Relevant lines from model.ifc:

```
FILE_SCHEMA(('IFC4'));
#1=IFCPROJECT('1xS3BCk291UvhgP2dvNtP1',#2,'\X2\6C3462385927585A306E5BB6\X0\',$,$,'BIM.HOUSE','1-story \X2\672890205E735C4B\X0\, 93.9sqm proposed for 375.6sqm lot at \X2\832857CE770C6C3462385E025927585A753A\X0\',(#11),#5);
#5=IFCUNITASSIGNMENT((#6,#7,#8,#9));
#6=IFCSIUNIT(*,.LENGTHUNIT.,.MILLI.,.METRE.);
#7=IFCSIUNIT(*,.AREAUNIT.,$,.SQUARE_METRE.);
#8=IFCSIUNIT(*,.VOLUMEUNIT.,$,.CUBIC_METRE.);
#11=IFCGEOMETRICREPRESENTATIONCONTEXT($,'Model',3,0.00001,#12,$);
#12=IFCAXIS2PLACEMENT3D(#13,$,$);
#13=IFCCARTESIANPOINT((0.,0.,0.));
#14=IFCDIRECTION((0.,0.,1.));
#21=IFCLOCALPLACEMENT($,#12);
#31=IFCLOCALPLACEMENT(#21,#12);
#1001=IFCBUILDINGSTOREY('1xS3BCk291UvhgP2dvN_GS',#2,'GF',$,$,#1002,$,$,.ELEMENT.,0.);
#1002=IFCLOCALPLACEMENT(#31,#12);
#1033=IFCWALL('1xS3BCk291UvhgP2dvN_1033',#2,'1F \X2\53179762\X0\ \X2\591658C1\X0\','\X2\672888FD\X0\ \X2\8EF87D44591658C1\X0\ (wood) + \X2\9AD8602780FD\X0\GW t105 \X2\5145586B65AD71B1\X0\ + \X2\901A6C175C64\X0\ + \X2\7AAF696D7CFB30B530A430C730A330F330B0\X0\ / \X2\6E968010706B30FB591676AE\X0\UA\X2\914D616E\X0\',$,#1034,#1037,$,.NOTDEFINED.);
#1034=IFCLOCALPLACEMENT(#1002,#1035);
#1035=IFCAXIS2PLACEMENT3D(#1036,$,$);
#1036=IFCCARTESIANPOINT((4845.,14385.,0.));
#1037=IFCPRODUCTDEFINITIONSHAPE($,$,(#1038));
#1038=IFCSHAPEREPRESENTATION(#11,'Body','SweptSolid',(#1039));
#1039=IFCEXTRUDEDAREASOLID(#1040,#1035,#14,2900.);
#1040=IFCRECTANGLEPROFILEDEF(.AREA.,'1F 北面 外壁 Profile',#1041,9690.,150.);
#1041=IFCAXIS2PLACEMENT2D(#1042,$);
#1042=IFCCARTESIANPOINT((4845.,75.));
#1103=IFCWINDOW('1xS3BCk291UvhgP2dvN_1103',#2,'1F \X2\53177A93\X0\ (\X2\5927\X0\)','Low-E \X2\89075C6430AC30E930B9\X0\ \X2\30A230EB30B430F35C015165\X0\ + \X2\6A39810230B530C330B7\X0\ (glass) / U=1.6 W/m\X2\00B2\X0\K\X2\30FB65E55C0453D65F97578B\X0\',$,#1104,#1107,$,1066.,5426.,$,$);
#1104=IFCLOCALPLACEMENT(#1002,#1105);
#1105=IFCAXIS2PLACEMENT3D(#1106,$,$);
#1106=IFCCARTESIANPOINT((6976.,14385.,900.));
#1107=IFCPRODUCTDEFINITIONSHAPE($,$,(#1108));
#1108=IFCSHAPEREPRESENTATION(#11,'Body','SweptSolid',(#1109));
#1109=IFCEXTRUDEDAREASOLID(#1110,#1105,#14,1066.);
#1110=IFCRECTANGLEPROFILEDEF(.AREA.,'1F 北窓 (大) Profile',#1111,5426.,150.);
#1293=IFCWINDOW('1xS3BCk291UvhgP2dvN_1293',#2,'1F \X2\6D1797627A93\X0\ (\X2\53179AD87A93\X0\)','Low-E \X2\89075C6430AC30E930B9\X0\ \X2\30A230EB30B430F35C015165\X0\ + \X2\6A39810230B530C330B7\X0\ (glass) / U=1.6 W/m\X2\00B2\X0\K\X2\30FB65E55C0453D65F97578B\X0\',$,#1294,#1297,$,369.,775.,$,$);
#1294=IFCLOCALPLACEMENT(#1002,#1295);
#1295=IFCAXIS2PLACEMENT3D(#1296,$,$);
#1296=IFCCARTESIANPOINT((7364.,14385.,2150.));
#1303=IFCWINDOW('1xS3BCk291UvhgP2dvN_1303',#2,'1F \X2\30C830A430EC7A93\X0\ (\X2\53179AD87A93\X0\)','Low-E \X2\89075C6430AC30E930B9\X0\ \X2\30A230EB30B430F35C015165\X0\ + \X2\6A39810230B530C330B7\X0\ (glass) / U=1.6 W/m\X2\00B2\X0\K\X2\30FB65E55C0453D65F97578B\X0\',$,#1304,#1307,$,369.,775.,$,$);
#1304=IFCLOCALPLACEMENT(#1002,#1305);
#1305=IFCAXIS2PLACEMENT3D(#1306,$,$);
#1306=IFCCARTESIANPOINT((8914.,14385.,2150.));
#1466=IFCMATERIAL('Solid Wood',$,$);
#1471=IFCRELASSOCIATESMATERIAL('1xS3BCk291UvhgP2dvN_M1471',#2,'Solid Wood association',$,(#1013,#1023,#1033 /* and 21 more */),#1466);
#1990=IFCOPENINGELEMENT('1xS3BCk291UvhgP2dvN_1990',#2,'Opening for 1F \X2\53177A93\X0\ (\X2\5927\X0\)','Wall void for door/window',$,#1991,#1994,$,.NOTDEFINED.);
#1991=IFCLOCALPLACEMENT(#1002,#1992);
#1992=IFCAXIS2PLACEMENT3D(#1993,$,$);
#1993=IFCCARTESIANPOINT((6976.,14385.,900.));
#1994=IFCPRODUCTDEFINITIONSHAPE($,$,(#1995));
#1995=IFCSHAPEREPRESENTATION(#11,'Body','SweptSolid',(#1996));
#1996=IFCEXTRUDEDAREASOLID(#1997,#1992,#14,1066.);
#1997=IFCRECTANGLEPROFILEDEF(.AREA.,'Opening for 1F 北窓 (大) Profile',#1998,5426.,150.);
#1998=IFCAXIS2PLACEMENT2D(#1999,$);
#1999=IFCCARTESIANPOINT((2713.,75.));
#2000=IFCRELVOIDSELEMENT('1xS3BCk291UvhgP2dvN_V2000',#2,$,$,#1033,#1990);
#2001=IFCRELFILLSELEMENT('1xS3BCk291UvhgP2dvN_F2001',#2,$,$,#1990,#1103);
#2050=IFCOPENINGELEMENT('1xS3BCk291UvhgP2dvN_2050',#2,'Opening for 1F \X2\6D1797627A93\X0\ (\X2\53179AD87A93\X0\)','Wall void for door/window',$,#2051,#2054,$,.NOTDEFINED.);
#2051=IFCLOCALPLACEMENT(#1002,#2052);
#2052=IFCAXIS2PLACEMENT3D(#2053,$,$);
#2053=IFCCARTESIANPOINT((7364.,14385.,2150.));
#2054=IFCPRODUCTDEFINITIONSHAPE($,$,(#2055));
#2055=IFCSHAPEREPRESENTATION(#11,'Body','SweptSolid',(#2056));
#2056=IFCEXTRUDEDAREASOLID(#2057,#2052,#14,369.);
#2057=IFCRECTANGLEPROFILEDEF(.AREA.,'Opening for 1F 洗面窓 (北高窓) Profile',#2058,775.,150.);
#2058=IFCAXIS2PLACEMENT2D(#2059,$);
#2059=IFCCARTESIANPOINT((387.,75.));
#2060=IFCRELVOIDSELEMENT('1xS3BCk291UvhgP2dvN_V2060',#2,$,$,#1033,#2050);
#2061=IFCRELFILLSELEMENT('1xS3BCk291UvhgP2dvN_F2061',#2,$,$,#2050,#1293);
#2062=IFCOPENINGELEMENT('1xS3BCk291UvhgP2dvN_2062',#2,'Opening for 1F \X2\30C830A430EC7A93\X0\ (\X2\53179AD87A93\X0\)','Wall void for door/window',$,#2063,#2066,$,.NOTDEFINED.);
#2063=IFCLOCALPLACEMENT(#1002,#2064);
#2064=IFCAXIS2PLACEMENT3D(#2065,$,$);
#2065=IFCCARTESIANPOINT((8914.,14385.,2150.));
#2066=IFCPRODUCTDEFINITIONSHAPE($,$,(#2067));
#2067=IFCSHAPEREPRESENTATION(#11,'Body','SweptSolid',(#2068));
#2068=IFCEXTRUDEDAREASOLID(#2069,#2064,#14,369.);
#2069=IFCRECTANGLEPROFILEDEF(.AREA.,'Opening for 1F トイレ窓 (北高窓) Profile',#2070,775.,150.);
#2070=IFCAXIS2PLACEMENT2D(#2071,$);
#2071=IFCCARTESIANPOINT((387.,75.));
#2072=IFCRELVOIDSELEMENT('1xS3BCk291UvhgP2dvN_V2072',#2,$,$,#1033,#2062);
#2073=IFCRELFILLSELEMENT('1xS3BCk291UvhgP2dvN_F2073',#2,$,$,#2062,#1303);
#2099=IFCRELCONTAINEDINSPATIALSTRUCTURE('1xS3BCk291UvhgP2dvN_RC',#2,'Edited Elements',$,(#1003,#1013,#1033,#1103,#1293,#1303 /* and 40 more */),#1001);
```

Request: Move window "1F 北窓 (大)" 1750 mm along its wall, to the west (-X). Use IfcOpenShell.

```python
import ifcopenshell
import ifcopenshell.api.geometry
import ifcopenshell.util.placement
import ifcopenshell.util.unit

model = ifcopenshell.open("model.ifc")
unit_scale = ifcopenshell.util.unit.calculate_unit_scale(model)

window = model.by_guid("1xS3BCk291UvhgP2dvN_1103")
opening = window.FillsVoids[0].RelatingOpeningElement
wall = opening.VoidsElements[0].RelatingBuildingElement

wall_matrix = ifcopenshell.util.placement.get_local_placement(wall.ObjectPlacement)
shift = wall_matrix[:3, 0] * -1.75 / unit_scale
before = ifcopenshell.util.placement.get_local_placement(window.ObjectPlacement)[:3, 3].copy()

# The window is not placed relative to its opening, so move both.
for product in (opening, window):
    matrix = ifcopenshell.util.placement.get_local_placement(product.ObjectPlacement)
    matrix[:3, 3] += shift
    ifcopenshell.api.geometry.edit_object_placement(model, product=product, matrix=matrix, is_si=False)

after = ifcopenshell.util.placement.get_local_placement(window.ObjectPlacement)[:3, 3]
print("window moved by", (after - before).round(3) + 0.0)

model.write("model_edited.ifc")
```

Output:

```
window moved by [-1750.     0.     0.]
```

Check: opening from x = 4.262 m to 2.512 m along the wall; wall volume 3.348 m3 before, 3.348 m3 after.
